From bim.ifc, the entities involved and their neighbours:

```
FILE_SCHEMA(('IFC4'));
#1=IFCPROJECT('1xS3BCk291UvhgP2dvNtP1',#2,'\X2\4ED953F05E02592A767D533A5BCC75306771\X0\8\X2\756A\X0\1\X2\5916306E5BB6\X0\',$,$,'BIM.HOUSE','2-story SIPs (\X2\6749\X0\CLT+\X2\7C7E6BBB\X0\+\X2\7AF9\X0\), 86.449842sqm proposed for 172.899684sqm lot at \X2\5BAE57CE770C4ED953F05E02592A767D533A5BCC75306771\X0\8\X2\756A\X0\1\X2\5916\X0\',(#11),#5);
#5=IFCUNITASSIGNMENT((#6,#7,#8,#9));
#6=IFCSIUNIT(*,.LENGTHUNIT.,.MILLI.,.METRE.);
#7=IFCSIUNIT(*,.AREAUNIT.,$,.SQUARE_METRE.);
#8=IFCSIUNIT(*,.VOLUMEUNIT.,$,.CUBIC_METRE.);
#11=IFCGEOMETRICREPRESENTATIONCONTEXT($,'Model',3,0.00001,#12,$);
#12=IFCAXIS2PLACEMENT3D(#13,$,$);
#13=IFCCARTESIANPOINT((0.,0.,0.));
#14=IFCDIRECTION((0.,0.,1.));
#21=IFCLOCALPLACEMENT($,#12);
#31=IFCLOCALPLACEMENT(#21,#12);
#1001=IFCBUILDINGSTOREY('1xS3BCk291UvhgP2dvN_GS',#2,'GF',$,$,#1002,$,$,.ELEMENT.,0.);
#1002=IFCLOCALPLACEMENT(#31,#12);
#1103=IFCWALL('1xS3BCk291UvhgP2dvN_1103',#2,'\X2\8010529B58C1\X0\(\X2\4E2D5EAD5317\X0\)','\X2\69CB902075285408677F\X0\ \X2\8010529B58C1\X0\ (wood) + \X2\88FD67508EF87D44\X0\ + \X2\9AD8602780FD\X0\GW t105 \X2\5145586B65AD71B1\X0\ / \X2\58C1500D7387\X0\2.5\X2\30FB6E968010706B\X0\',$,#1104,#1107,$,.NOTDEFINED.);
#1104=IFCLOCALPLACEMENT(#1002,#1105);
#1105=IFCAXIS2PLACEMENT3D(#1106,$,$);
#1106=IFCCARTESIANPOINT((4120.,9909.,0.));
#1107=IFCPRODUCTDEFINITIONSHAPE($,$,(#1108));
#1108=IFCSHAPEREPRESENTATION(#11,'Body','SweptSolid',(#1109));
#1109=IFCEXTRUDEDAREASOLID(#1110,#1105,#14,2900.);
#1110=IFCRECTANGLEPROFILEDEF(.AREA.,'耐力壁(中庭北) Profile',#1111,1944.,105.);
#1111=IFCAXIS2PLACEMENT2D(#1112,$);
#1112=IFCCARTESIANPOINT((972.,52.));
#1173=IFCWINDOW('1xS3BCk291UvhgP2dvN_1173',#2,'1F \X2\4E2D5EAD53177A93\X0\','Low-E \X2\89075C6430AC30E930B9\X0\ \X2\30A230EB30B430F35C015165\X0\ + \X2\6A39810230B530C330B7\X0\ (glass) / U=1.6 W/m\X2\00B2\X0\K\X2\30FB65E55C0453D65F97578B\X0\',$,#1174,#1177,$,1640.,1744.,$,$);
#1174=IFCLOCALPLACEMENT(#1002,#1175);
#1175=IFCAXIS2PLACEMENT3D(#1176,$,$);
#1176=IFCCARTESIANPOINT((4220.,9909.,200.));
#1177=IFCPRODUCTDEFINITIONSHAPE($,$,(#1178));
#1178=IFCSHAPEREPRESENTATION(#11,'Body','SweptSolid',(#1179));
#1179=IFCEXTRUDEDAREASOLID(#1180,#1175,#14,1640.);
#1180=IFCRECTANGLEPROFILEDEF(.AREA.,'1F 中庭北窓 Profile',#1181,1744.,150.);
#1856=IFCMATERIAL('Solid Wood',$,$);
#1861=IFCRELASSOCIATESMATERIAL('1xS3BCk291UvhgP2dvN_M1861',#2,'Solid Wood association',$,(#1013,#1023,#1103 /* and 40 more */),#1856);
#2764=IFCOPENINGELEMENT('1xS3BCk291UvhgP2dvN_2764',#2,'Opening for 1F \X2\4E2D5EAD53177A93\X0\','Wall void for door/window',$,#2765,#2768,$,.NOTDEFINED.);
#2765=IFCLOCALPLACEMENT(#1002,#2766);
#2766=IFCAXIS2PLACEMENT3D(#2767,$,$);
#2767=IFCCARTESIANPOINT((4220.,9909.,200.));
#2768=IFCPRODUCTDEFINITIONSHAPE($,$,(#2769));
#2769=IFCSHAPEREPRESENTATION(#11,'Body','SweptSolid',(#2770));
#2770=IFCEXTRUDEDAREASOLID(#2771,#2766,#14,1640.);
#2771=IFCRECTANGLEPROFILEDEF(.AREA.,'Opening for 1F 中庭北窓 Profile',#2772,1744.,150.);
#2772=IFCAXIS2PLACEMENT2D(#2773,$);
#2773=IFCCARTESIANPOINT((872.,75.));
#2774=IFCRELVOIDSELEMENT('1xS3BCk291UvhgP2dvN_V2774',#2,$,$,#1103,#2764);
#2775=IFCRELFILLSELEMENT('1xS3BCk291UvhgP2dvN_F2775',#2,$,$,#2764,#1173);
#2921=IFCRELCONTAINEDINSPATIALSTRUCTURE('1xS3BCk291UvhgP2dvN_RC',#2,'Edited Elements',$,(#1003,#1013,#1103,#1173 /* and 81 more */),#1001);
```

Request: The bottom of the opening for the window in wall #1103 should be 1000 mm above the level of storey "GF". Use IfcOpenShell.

```python
import numpy as np
import ifcopenshell
import ifcopenshell.api.geometry
import ifcopenshell.geom
import ifcopenshell.util.element
import ifcopenshell.util.placement
import ifcopenshell.util.shape
import ifcopenshell.util.unit

model = ifcopenshell.open("bim.ifc")
unit_scale = ifcopenshell.util.unit.calculate_unit_scale(model)

window = model.by_id(1173)
opening = window.FillsVoids[0].RelatingOpeningElement
storey = ifcopenshell.util.element.get_container(window, ifc_class="IfcBuildingStorey")
level = ifcopenshell.util.placement.get_local_placement(storey.ObjectPlacement)[2, 3]

# The opening's origin need not be at the sill, so measure its lowest point.
shape = ifcopenshell.geom.create_shape(ifcopenshell.geom.settings(), opening)
bottom = ifcopenshell.util.shape.get_shape_bottom_elevation(shape, shape.geometry) / unit_scale
dz = level + 1000.0 - bottom

shift = np.array([0.0, 0.0, dz])
# The window is not placed relative to its opening, so move both.
for product in (opening, window):
    matrix = ifcopenshell.util.placement.get_local_placement(product.ObjectPlacement)
    matrix[:3, 3] += shift
    ifcopenshell.api.geometry.edit_object_placement(model, product=product, matrix=matrix, is_si=False)

print(f"moved by {dz * unit_scale:+.3f} m")

model.write("bim-out.ifc")
```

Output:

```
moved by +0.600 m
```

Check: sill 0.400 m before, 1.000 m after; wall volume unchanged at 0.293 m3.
